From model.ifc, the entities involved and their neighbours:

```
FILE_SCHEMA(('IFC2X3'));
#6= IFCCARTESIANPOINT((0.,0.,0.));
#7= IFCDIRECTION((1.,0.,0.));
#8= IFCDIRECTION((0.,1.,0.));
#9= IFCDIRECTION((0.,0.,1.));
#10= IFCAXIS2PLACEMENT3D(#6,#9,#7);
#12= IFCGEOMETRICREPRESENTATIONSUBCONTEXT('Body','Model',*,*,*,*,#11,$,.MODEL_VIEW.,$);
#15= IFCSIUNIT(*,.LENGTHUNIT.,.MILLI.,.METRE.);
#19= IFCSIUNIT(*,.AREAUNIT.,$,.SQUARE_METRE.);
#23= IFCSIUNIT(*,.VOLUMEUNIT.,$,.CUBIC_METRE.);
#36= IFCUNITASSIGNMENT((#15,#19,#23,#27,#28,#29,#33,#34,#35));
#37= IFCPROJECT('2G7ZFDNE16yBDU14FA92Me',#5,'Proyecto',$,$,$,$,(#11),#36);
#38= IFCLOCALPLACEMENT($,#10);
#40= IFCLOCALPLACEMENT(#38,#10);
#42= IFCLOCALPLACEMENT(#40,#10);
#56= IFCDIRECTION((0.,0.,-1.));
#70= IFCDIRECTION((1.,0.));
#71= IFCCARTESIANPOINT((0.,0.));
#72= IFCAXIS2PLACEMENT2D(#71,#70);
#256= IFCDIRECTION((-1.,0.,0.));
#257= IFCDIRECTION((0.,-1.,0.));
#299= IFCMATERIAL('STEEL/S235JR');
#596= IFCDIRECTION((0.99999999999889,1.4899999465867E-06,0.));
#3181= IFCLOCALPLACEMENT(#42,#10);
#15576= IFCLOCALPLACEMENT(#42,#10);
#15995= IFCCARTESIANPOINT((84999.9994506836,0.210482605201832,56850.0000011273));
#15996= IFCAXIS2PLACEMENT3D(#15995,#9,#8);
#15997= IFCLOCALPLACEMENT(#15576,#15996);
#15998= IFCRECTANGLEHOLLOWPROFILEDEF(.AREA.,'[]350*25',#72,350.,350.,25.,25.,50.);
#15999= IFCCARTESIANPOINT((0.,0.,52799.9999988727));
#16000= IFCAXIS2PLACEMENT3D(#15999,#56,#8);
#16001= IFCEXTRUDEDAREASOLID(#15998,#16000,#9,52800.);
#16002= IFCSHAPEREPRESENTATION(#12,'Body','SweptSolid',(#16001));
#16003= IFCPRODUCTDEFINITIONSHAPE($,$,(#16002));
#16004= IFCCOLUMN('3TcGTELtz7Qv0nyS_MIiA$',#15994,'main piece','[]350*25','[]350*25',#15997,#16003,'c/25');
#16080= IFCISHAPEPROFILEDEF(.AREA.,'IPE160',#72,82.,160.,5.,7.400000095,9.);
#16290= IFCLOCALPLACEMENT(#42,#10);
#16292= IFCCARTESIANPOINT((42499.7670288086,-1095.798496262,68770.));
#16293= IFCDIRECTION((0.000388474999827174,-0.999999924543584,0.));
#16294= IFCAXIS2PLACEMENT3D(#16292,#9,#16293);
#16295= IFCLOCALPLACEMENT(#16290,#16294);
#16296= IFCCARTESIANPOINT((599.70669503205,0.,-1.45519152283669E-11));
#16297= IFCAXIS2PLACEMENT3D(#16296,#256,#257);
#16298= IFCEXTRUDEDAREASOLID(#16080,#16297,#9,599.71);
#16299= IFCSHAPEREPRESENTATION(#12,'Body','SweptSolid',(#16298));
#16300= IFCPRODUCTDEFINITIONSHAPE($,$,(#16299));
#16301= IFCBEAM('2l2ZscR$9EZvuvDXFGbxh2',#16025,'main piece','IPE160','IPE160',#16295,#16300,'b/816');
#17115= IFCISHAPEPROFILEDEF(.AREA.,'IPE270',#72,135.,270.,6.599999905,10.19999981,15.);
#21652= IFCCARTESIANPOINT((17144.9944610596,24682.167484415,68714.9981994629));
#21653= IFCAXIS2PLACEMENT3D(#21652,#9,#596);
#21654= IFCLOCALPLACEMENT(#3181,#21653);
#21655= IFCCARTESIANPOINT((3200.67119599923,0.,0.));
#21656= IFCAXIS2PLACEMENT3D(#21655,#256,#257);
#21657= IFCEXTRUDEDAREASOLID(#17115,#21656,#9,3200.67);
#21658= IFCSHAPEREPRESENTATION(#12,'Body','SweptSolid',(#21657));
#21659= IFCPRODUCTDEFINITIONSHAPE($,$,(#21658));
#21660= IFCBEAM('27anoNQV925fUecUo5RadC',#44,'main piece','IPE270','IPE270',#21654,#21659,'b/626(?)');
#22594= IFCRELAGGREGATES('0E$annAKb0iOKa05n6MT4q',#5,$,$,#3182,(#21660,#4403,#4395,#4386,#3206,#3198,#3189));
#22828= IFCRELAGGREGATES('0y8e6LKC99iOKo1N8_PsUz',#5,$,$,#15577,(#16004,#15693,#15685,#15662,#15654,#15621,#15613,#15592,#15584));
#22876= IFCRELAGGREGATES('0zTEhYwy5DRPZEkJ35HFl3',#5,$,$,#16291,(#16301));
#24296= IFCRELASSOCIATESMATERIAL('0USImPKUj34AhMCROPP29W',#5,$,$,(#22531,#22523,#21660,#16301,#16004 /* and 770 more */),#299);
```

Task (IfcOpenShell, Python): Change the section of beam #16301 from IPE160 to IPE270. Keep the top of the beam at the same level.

```python
import ifcopenshell
import ifcopenshell.util.element
import ifcopenshell.util.representation

model = ifcopenshell.open("model.ifc")

member = model.by_id(16301)
source = next(p for p in model.by_type("IfcIShapeProfileDef") if p.ProfileName == "IPE270")

body = ifcopenshell.util.representation.get_representation(member, "Model", "Body")
solid = body.Items[0]
old_profile = solid.SweptArea

# Copy the section's sizes but keep this member's own profile position.
profile = ifcopenshell.util.element.copy(model, source)
# Profiles are centred, so shift by half the change in depth to hold the top.
shift = (old_profile.OverallDepth - profile.OverallDepth) / 2
x, y = old_profile.Position.Location.Coordinates
up = (0.0, 1.0)  # upwards, in the solid's own plane
location = model.createIfcCartesianPoint((x + up[0] * shift, y + up[1] * shift))
profile.Position = model.createIfcAxis2Placement2D(location, old_profile.Position.RefDirection)
solid.SweptArea = profile
if not model.get_total_inverses(old_profile):
    ifcopenshell.util.element.remove_deep2(model, old_profile)
member.Description = member.Description.replace("IPE160", "IPE270")
member.ObjectType = member.ObjectType.replace("IPE160", "IPE270")

print(solid.SweptArea)

model.write("model_v2.ifc")
```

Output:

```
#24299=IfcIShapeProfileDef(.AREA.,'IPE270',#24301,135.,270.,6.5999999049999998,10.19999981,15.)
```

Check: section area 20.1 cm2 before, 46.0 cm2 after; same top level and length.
